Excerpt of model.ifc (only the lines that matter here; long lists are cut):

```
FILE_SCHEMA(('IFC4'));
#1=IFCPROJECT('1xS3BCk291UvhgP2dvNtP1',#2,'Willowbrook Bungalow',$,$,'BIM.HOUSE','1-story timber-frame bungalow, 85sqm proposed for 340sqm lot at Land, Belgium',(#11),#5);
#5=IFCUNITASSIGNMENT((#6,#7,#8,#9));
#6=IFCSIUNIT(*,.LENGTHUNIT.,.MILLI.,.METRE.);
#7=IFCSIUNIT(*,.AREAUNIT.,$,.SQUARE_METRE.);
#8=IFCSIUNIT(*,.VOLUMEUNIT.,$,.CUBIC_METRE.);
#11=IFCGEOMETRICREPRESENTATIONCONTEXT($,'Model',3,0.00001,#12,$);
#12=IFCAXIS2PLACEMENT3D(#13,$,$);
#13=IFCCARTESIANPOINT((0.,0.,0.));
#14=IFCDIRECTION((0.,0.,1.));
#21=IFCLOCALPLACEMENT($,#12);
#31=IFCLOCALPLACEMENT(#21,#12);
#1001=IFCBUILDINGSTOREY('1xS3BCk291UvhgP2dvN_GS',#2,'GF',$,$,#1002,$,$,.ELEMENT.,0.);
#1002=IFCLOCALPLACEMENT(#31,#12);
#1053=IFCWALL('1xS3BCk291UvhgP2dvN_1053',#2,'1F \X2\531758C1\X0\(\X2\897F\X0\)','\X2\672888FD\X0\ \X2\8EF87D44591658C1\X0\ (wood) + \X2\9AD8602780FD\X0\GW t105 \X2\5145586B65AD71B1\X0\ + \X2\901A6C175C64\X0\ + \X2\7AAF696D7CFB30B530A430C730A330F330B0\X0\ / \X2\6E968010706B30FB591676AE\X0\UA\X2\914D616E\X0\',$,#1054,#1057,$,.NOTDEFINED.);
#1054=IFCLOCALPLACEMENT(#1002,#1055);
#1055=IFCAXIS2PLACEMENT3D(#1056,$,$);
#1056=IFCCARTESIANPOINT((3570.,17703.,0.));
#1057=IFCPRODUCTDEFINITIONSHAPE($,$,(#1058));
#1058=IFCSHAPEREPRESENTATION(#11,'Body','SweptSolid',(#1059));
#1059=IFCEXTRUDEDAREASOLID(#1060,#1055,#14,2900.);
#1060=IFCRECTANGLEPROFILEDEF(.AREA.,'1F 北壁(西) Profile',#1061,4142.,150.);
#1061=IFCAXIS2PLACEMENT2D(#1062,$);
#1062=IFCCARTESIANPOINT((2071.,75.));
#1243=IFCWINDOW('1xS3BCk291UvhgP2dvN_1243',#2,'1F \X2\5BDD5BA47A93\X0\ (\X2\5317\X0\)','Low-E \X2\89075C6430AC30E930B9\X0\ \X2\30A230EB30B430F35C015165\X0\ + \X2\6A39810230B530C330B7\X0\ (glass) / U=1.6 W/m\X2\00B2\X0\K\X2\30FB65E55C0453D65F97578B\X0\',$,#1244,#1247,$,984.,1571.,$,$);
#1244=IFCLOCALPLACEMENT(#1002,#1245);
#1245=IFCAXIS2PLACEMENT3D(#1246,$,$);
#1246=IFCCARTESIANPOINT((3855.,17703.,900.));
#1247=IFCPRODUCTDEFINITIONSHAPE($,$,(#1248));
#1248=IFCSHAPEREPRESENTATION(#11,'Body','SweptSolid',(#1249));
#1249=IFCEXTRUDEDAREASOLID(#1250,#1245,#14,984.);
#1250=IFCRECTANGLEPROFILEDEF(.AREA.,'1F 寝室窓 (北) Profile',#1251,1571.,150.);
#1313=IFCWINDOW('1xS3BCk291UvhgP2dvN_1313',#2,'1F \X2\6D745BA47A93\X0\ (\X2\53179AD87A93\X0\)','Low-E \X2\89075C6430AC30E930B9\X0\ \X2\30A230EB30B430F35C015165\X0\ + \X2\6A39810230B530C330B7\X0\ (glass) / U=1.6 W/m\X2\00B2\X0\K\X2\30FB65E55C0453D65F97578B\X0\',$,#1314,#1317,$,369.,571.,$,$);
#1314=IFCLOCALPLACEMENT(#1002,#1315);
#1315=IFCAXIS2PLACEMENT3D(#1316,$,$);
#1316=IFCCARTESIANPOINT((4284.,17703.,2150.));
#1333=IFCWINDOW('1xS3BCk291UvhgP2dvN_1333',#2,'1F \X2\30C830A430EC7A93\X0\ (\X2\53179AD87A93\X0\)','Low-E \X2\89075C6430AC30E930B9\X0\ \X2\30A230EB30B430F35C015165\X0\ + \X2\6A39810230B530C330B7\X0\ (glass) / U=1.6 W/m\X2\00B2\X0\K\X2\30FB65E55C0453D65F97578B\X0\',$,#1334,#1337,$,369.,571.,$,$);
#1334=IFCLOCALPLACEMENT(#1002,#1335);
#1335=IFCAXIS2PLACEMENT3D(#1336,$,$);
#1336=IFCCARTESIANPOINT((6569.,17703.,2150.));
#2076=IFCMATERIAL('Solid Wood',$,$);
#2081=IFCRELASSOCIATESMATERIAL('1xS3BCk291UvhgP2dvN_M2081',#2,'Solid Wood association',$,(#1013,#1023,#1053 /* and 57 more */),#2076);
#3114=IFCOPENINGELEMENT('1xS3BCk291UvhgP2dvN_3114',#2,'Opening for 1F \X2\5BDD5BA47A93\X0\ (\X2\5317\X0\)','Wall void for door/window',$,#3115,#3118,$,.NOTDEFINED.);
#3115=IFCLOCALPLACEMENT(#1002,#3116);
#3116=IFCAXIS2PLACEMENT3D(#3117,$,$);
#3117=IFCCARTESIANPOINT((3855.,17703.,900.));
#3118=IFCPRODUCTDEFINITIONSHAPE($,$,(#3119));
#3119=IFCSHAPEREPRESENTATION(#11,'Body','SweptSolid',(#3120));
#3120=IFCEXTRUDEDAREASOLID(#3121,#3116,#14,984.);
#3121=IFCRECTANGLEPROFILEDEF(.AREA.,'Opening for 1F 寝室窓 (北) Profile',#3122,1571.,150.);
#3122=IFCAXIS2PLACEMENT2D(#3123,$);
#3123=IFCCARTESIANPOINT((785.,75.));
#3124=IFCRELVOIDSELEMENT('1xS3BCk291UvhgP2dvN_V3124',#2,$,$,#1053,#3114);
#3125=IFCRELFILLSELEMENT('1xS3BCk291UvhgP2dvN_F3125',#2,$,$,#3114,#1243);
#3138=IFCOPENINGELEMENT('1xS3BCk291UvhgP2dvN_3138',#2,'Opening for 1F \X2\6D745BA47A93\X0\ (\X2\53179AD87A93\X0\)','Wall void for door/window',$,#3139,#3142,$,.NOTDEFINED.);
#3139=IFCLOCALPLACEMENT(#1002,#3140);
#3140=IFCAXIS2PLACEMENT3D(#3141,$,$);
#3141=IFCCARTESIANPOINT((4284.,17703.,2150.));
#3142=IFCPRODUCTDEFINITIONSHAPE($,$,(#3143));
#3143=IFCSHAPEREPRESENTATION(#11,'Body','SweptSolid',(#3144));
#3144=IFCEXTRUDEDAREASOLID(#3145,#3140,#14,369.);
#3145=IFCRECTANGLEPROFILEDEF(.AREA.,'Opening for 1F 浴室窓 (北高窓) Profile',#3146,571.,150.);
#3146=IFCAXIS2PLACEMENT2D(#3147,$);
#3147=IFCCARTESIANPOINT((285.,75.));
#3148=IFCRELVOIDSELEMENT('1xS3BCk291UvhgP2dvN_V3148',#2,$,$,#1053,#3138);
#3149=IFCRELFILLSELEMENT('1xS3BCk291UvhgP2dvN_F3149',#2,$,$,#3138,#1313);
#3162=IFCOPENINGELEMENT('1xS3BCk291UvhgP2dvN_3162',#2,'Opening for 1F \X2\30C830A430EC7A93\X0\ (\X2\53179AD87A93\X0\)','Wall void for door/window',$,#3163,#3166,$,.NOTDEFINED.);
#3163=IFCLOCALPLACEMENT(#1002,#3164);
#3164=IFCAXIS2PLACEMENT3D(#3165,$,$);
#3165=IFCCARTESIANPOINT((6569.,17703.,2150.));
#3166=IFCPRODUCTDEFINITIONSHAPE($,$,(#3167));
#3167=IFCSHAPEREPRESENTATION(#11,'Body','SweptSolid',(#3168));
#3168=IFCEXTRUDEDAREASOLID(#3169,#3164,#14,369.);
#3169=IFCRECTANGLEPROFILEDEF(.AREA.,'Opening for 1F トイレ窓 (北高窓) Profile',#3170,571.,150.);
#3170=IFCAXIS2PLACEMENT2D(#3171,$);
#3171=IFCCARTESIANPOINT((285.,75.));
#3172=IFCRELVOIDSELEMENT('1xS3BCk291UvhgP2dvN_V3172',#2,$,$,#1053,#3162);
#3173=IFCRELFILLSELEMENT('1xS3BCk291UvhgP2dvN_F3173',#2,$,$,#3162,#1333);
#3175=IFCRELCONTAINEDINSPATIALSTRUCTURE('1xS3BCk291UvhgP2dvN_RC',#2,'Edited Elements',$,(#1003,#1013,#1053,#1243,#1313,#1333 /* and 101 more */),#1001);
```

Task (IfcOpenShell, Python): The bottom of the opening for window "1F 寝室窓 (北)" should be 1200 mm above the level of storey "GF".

```python
import numpy as np
import ifcopenshell
import ifcopenshell.api.geometry
import ifcopenshell.geom
import ifcopenshell.util.element
import ifcopenshell.util.placement
import ifcopenshell.util.shape
import ifcopenshell.util.unit

model = ifcopenshell.open("model.ifc")
unit_scale = ifcopenshell.util.unit.calculate_unit_scale(model)

window = model.by_guid("1xS3BCk291UvhgP2dvN_1243")
opening = window.FillsVoids[0].RelatingOpeningElement
storey = ifcopenshell.util.element.get_container(window, ifc_class="IfcBuildingStorey")
level = ifcopenshell.util.placement.get_local_placement(storey.ObjectPlacement)[2, 3]

# The opening's origin need not be at the sill, so measure its lowest point.
shape = ifcopenshell.geom.create_shape(ifcopenshell.geom.settings(), opening)
bottom = ifcopenshell.util.shape.get_shape_bottom_elevation(shape, shape.geometry) / unit_scale
dz = level + 1200.0 - bottom

shift = np.array([0.0, 0.0, dz])
# The window is not placed relative to its opening, so move both.
for product in (opening, window):
    matrix = ifcopenshell.util.placement.get_local_placement(product.ObjectPlacement)
    matrix[:3, 3] += shift
    ifcopenshell.api.geometry.edit_object_placement(model, product=product, matrix=matrix, is_si=False)

print(f"moved by {dz * unit_scale:+.3f} m")

model.write("model-out.ifc")
```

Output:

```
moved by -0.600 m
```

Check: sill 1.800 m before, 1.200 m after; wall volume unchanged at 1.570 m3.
